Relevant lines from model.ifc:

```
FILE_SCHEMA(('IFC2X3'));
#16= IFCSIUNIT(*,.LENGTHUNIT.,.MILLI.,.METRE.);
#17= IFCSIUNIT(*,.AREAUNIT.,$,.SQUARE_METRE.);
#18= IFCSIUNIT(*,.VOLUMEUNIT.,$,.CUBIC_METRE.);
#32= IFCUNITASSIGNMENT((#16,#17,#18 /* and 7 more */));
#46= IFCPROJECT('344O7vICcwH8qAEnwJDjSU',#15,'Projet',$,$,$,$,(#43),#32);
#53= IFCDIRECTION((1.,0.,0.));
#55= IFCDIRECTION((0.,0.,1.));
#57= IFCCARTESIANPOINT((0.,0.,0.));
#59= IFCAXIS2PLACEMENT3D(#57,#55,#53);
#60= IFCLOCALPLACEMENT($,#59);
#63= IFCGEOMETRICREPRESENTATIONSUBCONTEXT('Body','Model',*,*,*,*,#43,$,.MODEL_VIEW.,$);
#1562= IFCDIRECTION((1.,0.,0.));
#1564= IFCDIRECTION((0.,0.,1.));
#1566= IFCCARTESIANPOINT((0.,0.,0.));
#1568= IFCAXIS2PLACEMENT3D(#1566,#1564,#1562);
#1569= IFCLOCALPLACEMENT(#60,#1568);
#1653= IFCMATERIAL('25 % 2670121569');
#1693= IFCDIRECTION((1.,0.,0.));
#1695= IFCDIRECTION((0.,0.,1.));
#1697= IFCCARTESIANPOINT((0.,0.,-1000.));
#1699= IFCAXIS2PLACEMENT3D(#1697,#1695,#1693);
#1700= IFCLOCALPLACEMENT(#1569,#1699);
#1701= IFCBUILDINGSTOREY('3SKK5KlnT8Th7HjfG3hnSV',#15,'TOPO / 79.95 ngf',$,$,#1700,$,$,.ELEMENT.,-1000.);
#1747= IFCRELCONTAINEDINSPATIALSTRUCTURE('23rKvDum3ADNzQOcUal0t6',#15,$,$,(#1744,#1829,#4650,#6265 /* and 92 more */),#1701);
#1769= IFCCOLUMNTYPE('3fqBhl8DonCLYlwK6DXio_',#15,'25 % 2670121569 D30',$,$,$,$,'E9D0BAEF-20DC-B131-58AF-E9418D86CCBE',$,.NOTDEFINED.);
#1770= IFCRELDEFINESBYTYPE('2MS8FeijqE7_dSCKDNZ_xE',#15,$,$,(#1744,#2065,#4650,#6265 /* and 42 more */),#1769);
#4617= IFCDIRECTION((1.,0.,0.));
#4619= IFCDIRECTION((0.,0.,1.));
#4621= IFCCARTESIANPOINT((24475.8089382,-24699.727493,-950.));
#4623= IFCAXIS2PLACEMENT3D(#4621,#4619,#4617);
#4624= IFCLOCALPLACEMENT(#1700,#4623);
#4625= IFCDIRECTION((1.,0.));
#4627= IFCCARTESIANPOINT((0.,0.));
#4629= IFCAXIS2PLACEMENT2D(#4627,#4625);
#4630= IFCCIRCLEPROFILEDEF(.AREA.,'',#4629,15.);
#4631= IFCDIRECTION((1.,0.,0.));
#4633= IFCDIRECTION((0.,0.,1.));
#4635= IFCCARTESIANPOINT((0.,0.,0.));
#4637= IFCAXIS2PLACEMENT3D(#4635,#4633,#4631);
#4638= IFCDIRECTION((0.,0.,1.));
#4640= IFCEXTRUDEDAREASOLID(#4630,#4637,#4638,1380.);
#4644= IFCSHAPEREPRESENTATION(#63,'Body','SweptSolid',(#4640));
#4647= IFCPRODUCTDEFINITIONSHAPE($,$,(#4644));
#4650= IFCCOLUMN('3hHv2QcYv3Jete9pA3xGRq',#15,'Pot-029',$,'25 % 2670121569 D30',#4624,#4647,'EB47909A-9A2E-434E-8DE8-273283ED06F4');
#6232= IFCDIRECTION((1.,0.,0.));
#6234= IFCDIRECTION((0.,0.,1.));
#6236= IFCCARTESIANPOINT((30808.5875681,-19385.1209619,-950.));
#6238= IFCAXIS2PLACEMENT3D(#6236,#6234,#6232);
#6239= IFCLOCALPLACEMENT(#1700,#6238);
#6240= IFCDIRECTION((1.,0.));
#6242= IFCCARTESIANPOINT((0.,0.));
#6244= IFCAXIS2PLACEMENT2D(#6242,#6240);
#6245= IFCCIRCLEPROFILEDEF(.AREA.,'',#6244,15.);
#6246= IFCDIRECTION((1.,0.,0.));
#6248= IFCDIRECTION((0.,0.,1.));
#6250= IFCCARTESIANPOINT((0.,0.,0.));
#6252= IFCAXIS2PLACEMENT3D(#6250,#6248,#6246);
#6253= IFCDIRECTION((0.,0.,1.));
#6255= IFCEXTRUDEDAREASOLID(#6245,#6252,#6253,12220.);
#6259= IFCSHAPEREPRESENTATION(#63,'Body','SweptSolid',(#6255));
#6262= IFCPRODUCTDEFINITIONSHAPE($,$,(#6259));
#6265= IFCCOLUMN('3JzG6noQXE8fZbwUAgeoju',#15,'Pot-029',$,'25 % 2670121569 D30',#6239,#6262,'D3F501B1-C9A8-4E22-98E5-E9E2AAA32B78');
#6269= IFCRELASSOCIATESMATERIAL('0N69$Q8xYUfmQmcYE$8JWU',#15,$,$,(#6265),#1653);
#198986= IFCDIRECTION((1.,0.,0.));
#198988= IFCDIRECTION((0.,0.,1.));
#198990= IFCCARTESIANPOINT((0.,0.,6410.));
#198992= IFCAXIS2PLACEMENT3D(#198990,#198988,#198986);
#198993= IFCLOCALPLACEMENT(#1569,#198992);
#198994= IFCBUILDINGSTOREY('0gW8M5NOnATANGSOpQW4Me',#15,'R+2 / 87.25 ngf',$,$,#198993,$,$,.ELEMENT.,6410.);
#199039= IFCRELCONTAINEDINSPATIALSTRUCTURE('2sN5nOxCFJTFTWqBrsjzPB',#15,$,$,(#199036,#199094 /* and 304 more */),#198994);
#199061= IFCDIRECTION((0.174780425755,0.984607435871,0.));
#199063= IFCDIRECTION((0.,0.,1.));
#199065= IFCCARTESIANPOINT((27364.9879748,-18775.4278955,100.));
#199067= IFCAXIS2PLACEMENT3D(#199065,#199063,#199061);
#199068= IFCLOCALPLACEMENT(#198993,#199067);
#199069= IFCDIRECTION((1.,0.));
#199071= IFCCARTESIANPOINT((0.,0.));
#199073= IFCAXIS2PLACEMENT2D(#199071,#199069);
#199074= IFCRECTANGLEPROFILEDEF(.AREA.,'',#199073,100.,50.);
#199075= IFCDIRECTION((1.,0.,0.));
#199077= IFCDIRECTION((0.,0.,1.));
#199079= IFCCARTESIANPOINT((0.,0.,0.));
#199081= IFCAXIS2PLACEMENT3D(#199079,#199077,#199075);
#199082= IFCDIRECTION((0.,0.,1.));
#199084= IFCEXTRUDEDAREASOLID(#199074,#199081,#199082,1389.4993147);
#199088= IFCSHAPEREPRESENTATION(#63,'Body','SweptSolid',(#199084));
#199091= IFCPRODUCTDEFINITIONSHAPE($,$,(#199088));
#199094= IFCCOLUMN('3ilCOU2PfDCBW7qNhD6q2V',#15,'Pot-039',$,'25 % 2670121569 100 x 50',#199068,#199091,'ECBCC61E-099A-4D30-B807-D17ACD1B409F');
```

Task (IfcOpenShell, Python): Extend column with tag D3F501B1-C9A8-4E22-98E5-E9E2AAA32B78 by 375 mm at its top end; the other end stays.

```python
import ifcopenshell
import ifcopenshell.util.representation
import ifcopenshell.util.unit

model = ifcopenshell.open("model.ifc")
unit_scale = ifcopenshell.util.unit.calculate_unit_scale(model)

member = model.by_id(6265)
change = 0.375 / unit_scale

# The extrusion runs towards the end named, so only its depth changes.
body = ifcopenshell.util.representation.get_representation(member, "Model", "Body")
solid = body.Items[0]
old_length = solid.Depth
solid.Depth += change

print(f"length {old_length:g} -> {solid.Depth:g}")

model.write("model_v2.ifc")
```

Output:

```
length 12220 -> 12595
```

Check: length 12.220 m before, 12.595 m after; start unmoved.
